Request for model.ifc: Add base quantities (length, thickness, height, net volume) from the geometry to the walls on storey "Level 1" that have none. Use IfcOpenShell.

First a look at what the model holds.

```python
import ifcopenshell
import ifcopenshell.util.element
import ifcopenshell.util.unit

model = ifcopenshell.open("model.ifc")
print(model.schema)
for unit_type in ("LENGTHUNIT", "AREAUNIT", "VOLUMEUNIT"):
    print(unit_type, ifcopenshell.util.unit.calculate_unit_scale(model, unit_type))
storey = next(s for s in model.by_type("IfcBuildingStorey") if s.Name == "Level 1")
walls = [e for e in ifcopenshell.util.element.get_decomposition(storey) if e.is_a("IfcWall")]
for e in sorted(walls, key=lambda e: e.id()):
    print(e.id(), e.is_a(), e.Name, list(ifcopenshell.util.element.get_psets(e, qtos_only=True)), sep=" | ")
```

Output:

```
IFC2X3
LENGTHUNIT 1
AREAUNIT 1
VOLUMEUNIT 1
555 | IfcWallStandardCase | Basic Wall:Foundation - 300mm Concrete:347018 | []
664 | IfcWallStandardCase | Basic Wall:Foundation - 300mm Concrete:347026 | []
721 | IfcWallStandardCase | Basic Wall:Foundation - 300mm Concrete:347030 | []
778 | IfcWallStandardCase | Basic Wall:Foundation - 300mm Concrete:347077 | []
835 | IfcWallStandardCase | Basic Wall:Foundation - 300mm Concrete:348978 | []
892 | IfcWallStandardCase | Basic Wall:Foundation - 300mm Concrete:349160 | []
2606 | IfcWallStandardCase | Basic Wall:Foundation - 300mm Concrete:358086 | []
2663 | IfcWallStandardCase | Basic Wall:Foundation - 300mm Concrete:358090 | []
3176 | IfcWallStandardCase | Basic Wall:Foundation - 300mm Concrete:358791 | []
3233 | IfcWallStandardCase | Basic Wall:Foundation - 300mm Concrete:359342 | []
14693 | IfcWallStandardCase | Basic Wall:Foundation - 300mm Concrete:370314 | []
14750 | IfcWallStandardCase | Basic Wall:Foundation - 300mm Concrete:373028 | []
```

```python
import ifcopenshell
import ifcopenshell.api.pset
import ifcopenshell.geom
import ifcopenshell.util.element
import ifcopenshell.util.shape
import ifcopenshell.util.unit

model = ifcopenshell.open("model.ifc")
unit_scale = ifcopenshell.util.unit.calculate_unit_scale(model)
volume_scale = ifcopenshell.util.unit.calculate_unit_scale(model, "VOLUMEUNIT")
settings = ifcopenshell.geom.settings()

storey = next(s for s in model.by_type("IfcBuildingStorey") if s.Name == "Level 1")
walls = [e for e in ifcopenshell.util.element.get_decomposition(storey) if e.is_a("IfcWall")]

for e in sorted(walls, key=lambda e: e.id()):
    if ifcopenshell.util.element.get_psets(e, qtos_only=True, should_inherit=False):
        continue
    # Geometry comes back in metres, in the element's own axes.
    shape = ifcopenshell.geom.create_shape(settings, e)
    values = {
        "Length": ifcopenshell.util.shape.get_x(shape.geometry) / unit_scale,
        "Width": ifcopenshell.util.shape.get_y(shape.geometry) / unit_scale,
        "Height": ifcopenshell.util.shape.get_z(shape.geometry) / unit_scale,
        "NetVolume": ifcopenshell.util.shape.get_volume(shape.geometry) / volume_scale,
    }
    qto = ifcopenshell.api.pset.add_qto(model, product=e, name="BaseQuantities")
    ifcopenshell.api.pset.edit_qto(model, qto=qto, properties=values)
    print(e.id(), {k: round(v, 3) for k, v in values.items()})

model.write("model_v2.ifc")
```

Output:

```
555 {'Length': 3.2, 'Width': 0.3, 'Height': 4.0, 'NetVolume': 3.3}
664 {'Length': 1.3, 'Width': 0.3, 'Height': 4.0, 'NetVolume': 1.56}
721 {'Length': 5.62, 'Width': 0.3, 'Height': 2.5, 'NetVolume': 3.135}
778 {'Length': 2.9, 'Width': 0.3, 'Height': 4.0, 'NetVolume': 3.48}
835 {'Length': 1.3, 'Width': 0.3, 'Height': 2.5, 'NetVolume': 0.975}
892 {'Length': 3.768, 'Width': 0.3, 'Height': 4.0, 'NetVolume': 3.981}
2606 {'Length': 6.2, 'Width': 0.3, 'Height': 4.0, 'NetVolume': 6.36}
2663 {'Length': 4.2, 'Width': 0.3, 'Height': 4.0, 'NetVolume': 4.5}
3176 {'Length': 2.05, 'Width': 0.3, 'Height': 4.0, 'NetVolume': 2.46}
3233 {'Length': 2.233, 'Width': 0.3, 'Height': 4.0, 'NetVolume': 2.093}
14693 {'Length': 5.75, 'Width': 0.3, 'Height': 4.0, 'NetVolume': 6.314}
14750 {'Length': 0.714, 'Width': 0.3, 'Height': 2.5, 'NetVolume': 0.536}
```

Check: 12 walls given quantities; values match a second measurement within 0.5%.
